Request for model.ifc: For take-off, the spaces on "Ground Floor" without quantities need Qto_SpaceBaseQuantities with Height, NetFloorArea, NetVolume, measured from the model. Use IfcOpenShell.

First a look at what the model holds.

```python
import ifcopenshell
import ifcopenshell.util.element
import ifcopenshell.util.unit

model = ifcopenshell.open("model.ifc")
print(model.schema)
for unit_type in ("LENGTHUNIT", "AREAUNIT", "VOLUMEUNIT"):
    print(unit_type, ifcopenshell.util.unit.calculate_unit_scale(model, unit_type))
storey = next(s for s in model.by_type("IfcBuildingStorey") if s.Name == "Ground Floor")
spaces = [e for e in ifcopenshell.util.element.get_decomposition(storey) if e.is_a("IfcSpace")]
for e in sorted(spaces, key=lambda e: e.id()):
    print(e.id(), e.is_a(), e.Name, list(ifcopenshell.util.element.get_psets(e, qtos_only=True)), sep=" | ")
```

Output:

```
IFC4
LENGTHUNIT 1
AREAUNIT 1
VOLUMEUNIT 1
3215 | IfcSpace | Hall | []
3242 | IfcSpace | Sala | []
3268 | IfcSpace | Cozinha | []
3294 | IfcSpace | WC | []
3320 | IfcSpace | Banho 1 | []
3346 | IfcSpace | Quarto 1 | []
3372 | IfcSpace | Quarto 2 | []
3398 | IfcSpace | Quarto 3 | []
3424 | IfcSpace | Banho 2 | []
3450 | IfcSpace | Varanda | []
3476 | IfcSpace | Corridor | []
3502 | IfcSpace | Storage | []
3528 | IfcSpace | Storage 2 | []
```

```python
import ifcopenshell
import ifcopenshell.api.pset
import ifcopenshell.geom
import ifcopenshell.util.element
import ifcopenshell.util.shape
import ifcopenshell.util.unit

model = ifcopenshell.open("model.ifc")
unit_scale = ifcopenshell.util.unit.calculate_unit_scale(model)
area_scale = ifcopenshell.util.unit.calculate_unit_scale(model, "AREAUNIT")
volume_scale = ifcopenshell.util.unit.calculate_unit_scale(model, "VOLUMEUNIT")
settings = ifcopenshell.geom.settings()

storey = next(s for s in model.by_type("IfcBuildingStorey") if s.Name == "Ground Floor")
spaces = [e for e in ifcopenshell.util.element.get_decomposition(storey) if e.is_a("IfcSpace")]

for e in sorted(spaces, key=lambda e: e.id()):
    if ifcopenshell.util.element.get_psets(e, qtos_only=True, should_inherit=False):
        continue
    # Geometry comes back in metres, in the element's own axes.
    shape = ifcopenshell.geom.create_shape(settings, e)
    values = {
        "Height": ifcopenshell.util.shape.get_z(shape.geometry) / unit_scale,
        "NetFloorArea": ifcopenshell.util.shape.get_footprint_area(shape.geometry) / area_scale,
        "NetVolume": ifcopenshell.util.shape.get_volume(shape.geometry) / volume_scale,
    }
    qto = ifcopenshell.api.pset.add_qto(model, product=e, name="Qto_SpaceBaseQuantities")
    ifcopenshell.api.pset.edit_qto(model, qto=qto, properties=values)
    print(e.id(), {k: round(v, 3) for k, v in values.items()})

model.write("model_v2.ifc")
```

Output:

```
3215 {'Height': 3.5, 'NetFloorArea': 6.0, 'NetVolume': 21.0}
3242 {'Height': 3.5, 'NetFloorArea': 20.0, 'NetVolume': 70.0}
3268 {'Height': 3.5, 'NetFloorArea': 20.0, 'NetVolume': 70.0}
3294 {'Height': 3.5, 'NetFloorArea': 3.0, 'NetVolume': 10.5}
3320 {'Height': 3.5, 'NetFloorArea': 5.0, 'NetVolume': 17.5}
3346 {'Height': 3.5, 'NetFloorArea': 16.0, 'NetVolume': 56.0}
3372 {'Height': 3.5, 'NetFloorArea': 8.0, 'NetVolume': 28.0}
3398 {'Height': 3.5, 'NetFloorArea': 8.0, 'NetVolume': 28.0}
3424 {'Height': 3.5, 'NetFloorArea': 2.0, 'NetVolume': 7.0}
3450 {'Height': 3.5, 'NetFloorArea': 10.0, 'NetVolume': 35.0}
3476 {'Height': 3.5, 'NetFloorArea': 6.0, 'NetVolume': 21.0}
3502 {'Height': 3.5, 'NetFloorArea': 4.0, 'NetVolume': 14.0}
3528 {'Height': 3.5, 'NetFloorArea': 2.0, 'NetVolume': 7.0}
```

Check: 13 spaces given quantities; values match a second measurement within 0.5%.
